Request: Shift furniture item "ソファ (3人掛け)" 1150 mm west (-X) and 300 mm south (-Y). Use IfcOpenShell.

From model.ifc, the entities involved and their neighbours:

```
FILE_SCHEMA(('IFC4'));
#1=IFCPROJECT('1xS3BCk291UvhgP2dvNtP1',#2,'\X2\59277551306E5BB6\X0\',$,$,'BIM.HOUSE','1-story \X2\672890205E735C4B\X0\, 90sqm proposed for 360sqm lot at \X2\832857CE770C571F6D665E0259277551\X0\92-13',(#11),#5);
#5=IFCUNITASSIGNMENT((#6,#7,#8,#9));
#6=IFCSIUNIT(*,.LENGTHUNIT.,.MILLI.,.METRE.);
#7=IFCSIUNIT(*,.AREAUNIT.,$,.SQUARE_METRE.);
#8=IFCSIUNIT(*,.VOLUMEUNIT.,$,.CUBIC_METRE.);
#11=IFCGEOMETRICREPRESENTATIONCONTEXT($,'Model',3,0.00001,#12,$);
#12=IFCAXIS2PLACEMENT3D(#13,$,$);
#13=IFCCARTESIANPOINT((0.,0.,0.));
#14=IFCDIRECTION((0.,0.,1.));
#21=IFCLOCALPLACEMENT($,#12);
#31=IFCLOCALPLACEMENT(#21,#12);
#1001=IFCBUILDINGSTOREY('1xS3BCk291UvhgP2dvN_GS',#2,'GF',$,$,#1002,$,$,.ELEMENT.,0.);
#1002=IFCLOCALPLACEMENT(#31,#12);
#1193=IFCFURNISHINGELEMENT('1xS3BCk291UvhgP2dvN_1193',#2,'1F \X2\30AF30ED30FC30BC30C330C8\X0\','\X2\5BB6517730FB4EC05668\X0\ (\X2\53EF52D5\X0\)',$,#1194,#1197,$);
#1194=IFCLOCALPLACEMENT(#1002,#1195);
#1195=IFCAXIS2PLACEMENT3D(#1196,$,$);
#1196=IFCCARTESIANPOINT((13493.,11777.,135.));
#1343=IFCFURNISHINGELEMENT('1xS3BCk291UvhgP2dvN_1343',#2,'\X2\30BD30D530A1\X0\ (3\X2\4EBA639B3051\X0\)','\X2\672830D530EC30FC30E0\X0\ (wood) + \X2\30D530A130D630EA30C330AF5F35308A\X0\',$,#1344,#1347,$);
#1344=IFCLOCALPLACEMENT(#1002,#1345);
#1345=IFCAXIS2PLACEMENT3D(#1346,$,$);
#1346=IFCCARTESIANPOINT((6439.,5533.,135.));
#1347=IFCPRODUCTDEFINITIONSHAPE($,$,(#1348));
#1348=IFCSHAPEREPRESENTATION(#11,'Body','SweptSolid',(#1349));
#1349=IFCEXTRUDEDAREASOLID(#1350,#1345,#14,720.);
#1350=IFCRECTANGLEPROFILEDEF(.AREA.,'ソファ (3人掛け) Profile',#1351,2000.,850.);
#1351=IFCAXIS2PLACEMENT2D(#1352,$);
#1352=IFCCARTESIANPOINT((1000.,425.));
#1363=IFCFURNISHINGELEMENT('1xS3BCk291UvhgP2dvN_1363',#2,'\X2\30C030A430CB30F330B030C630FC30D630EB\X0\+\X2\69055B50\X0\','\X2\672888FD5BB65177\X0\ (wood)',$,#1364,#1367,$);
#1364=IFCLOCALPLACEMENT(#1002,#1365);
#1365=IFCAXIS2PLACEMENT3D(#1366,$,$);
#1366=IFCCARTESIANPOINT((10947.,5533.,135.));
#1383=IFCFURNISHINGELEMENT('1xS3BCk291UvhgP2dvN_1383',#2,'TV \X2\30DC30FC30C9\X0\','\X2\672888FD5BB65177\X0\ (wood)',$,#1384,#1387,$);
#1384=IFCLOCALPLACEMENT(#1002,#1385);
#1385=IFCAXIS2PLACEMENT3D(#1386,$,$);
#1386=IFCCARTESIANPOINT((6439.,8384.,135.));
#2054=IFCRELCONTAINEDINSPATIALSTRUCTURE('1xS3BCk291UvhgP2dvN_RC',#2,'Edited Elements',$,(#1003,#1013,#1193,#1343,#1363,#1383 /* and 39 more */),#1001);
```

```python
import ifcopenshell
import ifcopenshell.api.geometry
import ifcopenshell.util.placement
import ifcopenshell.util.unit

model = ifcopenshell.open("model.ifc")
unit_scale = ifcopenshell.util.unit.calculate_unit_scale(model)

item = model.by_id(1343)
matrix = ifcopenshell.util.placement.get_local_placement(item.ObjectPlacement)
matrix[0, 3] -= 1.15 / unit_scale
matrix[1, 3] -= 0.3 / unit_scale
ifcopenshell.api.geometry.edit_object_placement(model, product=item, matrix=matrix, is_si=False)

print(ifcopenshell.util.placement.get_local_placement(item.ObjectPlacement).round(3) + 0.0)

model.write("model_rev.ifc")
```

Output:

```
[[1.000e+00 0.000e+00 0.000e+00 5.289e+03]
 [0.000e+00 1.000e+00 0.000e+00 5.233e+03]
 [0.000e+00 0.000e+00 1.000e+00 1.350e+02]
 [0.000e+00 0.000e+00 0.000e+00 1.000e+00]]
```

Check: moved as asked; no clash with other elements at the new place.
